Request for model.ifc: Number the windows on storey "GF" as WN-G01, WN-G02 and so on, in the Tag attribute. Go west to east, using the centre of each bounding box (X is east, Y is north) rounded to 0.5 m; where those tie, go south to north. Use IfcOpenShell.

First a look at what the model holds.

```python
import ifcopenshell
import ifcopenshell.util.element
import ifcopenshell.util.placement

model = ifcopenshell.open("model.ifc")
print(model.schema)
storey = next(s for s in model.by_type("IfcBuildingStorey") if s.Name == "GF")
windows = [e for e in ifcopenshell.util.element.get_decomposition(storey) if e.is_a("IfcWindow")]
for e in sorted(windows, key=lambda e: e.id()):
    origin = ifcopenshell.util.placement.get_local_placement(e.ObjectPlacement)[:3, 3]
    print(e.id(), e.Tag, e.Name, origin.round(2) + 0.0, sep=" | ")
```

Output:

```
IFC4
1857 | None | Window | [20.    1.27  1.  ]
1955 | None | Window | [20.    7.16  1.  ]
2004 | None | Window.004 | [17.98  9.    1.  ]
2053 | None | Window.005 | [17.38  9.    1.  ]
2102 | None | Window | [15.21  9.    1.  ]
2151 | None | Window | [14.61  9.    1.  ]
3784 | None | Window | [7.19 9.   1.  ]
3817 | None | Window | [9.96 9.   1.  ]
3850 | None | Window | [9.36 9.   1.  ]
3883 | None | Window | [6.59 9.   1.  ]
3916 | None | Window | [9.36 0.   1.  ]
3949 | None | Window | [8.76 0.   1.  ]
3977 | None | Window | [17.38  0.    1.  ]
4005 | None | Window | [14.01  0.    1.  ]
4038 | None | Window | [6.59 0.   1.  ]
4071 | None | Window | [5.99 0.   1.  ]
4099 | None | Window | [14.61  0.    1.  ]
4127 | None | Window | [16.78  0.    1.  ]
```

```python
import ifcopenshell
import ifcopenshell.geom
import ifcopenshell.util.element
import ifcopenshell.util.shape

model = ifcopenshell.open("model.ifc")
settings = ifcopenshell.geom.settings()
settings.set("use-world-coords", True)


def centre(element):
    shape = ifcopenshell.geom.create_shape(settings, element)
    return ifcopenshell.util.shape.get_bbox_centroid(shape.geometry)


storey = next(s for s in model.by_type("IfcBuildingStorey") if s.Name == "GF")
windows = [e for e in ifcopenshell.util.element.get_decomposition(storey) if e.is_a("IfcWindow")]

# Insertion points can sit at a corner or the storey origin, so sort by the geometry (in metres).
centres = {e: centre(e) for e in windows}
windows.sort(key=lambda e: (round(centres[e][0] / 0.5), centres[e][1]))

for i, e in enumerate(windows, start=1):
    number = f"WN-G{i:02d}"
    e.Tag = number
    print(e.id(), number)

model.write("model_rev.ifc")
```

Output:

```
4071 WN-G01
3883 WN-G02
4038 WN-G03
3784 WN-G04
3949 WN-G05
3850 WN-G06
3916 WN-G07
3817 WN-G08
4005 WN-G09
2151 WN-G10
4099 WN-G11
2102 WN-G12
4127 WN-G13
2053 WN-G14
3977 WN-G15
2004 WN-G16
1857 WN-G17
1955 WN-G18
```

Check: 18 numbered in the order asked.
